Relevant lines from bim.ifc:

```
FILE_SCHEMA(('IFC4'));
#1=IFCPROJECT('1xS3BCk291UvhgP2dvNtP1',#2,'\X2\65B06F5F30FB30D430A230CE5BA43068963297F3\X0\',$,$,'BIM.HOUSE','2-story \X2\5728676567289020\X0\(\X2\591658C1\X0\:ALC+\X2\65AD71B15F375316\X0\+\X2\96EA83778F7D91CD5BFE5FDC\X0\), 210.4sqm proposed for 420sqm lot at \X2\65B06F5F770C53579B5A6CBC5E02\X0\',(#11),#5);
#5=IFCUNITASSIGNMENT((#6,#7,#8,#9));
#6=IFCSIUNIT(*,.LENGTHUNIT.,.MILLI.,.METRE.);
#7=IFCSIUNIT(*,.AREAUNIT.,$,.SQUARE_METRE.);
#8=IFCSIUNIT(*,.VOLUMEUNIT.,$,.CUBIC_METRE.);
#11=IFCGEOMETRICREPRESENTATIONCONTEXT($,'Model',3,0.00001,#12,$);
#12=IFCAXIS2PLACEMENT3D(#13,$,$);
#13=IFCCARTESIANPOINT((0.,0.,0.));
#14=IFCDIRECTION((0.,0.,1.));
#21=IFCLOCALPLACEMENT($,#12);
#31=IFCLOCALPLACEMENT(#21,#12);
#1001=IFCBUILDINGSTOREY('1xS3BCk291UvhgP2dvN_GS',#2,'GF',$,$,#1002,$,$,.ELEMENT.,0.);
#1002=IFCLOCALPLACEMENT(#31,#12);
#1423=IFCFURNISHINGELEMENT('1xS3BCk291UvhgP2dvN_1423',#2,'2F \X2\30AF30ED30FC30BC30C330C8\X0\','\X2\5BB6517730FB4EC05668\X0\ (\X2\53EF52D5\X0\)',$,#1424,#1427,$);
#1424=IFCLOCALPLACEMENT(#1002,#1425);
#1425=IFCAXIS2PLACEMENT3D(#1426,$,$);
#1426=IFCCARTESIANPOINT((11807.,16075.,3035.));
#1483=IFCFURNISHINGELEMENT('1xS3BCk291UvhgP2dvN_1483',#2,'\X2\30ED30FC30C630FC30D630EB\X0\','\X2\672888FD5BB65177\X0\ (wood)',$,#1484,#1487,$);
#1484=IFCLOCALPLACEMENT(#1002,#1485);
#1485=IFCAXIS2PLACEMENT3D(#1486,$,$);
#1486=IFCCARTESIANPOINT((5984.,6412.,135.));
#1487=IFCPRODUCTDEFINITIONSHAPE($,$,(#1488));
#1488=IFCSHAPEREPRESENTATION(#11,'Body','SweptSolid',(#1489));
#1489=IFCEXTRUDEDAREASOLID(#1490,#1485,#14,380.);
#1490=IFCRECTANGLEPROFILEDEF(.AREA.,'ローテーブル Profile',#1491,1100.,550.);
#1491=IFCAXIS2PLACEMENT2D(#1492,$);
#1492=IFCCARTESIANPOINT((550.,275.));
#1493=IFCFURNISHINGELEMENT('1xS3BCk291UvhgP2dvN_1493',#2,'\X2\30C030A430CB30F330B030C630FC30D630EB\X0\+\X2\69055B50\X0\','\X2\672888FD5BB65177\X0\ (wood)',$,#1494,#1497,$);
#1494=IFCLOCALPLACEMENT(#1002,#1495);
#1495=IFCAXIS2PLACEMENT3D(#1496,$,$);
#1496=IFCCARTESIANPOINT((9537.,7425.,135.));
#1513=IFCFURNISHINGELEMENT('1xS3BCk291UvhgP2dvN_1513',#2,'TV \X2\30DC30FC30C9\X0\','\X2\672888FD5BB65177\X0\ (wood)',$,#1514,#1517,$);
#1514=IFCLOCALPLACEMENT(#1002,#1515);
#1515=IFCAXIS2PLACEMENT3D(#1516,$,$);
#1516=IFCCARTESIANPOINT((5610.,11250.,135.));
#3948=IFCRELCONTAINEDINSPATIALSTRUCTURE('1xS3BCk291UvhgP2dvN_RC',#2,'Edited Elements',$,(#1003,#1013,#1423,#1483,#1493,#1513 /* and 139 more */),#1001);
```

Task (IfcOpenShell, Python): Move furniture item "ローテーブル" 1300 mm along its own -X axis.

```python
import ifcopenshell
import ifcopenshell.api.geometry
import ifcopenshell.util.placement

model = ifcopenshell.open("bim.ifc")

item = model.by_guid("1xS3BCk291UvhgP2dvN_1483")
matrix = ifcopenshell.util.placement.get_local_placement(item.ObjectPlacement)
matrix[:3, 3] -= matrix[:3, 0] * 1300.0
ifcopenshell.api.geometry.edit_object_placement(model, product=item, matrix=matrix, is_si=False)

print(ifcopenshell.util.placement.get_local_placement(item.ObjectPlacement).round(3) + 0.0)

model.write("bim_rev.ifc")
```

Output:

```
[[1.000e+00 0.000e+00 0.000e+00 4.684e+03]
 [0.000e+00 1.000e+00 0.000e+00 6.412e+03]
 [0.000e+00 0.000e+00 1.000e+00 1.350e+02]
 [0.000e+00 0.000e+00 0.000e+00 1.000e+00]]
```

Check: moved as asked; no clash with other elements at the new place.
